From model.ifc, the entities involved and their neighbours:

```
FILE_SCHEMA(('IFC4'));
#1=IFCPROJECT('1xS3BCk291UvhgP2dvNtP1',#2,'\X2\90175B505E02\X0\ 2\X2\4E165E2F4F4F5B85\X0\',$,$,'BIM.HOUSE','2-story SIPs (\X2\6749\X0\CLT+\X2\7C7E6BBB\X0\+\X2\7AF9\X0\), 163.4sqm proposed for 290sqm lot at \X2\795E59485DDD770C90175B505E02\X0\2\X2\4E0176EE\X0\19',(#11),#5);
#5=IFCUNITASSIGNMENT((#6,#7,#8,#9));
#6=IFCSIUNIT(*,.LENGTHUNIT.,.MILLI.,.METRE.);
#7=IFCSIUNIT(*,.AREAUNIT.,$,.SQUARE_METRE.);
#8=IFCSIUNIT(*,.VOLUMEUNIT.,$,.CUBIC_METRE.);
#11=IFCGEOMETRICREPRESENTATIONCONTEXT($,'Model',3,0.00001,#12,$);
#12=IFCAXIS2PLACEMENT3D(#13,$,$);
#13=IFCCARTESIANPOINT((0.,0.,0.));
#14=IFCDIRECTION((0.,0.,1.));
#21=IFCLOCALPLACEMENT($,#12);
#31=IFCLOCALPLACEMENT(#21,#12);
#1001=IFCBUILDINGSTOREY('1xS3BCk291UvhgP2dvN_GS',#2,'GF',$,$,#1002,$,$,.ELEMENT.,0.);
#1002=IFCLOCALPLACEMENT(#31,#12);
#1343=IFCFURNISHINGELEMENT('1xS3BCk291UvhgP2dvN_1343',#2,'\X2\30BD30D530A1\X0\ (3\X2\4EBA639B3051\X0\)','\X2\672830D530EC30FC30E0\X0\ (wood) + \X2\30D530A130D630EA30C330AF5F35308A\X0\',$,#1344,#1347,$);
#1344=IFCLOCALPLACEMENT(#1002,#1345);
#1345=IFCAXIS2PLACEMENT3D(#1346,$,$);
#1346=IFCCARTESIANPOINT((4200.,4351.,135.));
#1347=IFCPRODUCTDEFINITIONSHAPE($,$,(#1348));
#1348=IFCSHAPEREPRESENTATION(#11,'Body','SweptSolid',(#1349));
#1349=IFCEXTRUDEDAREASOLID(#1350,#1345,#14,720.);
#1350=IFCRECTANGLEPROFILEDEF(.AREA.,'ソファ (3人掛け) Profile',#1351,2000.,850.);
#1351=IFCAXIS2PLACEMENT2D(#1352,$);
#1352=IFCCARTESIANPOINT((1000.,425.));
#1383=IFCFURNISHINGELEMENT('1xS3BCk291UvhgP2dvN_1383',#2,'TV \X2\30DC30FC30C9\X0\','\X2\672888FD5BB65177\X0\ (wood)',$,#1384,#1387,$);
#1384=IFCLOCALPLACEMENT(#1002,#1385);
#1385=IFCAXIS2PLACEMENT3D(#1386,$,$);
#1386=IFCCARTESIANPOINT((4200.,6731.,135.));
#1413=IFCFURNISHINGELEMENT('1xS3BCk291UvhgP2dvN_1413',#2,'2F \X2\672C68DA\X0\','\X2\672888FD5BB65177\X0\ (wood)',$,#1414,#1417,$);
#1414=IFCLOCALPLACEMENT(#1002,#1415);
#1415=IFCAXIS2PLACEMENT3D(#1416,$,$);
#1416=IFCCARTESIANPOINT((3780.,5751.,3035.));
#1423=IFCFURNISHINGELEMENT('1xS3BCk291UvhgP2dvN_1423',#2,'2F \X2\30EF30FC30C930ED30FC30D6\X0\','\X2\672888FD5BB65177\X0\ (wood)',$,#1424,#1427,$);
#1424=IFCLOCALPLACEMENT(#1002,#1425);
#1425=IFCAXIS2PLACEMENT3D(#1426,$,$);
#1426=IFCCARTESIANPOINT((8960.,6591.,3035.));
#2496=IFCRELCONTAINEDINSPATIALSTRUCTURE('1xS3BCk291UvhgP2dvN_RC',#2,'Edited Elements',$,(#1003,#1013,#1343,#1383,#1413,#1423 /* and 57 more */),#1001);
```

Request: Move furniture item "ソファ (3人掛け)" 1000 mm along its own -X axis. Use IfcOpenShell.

```python
import ifcopenshell
import ifcopenshell.api.geometry
import ifcopenshell.util.placement
import ifcopenshell.util.unit

model = ifcopenshell.open("model.ifc")
unit_scale = ifcopenshell.util.unit.calculate_unit_scale(model)

item = model.by_guid("1xS3BCk291UvhgP2dvN_1343")
matrix = ifcopenshell.util.placement.get_local_placement(item.ObjectPlacement)
matrix[:3, 3] -= matrix[:3, 0] * 1 / unit_scale
ifcopenshell.api.geometry.edit_object_placement(model, product=item, matrix=matrix, is_si=False)

print(ifcopenshell.util.placement.get_local_placement(item.ObjectPlacement).round(3) + 0.0)

model.write("model_updated.ifc")
```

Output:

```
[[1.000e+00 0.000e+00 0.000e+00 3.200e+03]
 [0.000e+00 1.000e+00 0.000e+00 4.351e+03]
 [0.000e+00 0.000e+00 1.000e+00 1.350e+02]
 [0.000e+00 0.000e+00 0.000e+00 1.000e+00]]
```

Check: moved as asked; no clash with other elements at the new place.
